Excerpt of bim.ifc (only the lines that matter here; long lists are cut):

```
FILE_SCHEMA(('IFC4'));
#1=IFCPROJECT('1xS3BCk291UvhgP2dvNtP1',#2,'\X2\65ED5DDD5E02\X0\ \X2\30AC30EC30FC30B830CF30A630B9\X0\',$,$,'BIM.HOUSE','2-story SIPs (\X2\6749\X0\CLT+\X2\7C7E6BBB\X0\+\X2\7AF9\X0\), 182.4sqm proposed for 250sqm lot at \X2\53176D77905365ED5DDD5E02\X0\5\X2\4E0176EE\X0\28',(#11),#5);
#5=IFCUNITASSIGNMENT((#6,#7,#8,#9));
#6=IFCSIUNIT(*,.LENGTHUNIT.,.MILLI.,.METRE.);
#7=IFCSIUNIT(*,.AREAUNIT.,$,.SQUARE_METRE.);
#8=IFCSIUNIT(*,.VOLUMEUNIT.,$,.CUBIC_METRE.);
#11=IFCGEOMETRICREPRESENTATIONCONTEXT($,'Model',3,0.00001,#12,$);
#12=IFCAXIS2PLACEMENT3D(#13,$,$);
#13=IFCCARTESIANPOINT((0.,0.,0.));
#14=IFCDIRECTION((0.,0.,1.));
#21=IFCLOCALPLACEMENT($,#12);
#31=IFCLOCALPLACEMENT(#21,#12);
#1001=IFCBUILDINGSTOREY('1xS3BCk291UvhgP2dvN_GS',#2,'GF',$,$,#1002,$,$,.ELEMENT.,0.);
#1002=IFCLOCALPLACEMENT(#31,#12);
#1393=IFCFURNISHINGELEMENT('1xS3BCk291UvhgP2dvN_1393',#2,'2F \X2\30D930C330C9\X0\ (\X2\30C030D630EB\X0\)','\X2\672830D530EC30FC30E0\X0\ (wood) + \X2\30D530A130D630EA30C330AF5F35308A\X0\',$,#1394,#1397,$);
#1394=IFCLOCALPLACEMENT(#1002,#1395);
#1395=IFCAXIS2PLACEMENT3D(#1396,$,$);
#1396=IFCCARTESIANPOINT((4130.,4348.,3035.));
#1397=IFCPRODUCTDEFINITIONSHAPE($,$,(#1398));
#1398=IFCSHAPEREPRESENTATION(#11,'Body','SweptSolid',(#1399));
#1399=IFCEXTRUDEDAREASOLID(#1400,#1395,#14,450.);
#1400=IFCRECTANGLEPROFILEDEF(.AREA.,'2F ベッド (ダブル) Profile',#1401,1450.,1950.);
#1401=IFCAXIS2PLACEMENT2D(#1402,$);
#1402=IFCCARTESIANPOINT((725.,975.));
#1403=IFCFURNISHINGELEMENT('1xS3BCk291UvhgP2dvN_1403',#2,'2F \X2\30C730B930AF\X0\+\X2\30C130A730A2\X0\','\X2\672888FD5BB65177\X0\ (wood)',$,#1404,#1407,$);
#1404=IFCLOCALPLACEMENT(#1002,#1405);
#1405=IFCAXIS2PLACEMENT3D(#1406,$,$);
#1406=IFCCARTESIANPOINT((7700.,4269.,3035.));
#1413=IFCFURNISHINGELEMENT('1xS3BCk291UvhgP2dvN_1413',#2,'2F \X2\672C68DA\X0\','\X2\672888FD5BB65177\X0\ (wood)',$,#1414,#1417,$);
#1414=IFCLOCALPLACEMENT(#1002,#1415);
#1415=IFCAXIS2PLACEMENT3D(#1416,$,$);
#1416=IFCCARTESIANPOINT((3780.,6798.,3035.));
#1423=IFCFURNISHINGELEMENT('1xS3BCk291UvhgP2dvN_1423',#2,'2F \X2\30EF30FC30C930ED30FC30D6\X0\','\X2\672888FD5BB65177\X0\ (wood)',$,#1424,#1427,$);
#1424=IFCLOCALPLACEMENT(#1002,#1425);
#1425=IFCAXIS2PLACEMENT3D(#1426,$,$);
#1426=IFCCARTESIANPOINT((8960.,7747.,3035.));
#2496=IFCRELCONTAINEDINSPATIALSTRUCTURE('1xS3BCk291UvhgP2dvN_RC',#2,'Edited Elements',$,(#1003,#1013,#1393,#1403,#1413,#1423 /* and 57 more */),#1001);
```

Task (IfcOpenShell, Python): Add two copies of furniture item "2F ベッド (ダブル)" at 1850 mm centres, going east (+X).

```python
import numpy as np
import ifcopenshell
import ifcopenshell.api.geometry
import ifcopenshell.api.root
import ifcopenshell.util.element
import ifcopenshell.util.placement

model = ifcopenshell.open("bim.ifc")


def reuse_history(source, copy):
    """copy_class also copies each property set's owner history, people and application; keep the originals."""
    for rel in copy.IsDefinedBy:
        if rel.is_a("IfcRelDefinesByProperties") and (history := rel.RelatingPropertyDefinition.OwnerHistory):
            rel.RelatingPropertyDefinition.OwnerHistory = source.OwnerHistory
            ifcopenshell.util.element.remove_deep2(model, history)


source = model.by_guid("1xS3BCk291UvhgP2dvN_1393")
base = ifcopenshell.util.placement.get_local_placement(source.ObjectPlacement)
step = np.array([1.0, 0.0, 0.0]) * 1850.0

for i in range(1, 3):
    copy = ifcopenshell.api.root.copy_class(model, product=source)
    copy.Representation = ifcopenshell.util.element.copy_deep(
        model, source.Representation, exclude=["IfcGeometricRepresentationContext", "IfcRepresentationMap"]
    )
    reuse_history(source, copy)
    matrix = base.copy()
    matrix[:3, 3] += i * step
    print("added at", matrix[:3, 3].round(3) + 0.0)
    ifcopenshell.api.geometry.edit_object_placement(model, product=copy, matrix=matrix, is_si=False)

model.write("bim_v2.ifc")
```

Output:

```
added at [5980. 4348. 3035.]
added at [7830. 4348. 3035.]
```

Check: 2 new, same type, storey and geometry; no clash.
